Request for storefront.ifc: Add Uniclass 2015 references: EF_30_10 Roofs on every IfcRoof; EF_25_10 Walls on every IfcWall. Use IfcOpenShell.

First a look at what the model holds.

```python
import ifcopenshell

model = ifcopenshell.open("storefront.ifc")
print(model.schema)
print("classifications:", [c.Name for c in model.by_type("IfcClassification")])
for ifc_class in ("IfcDoor", "IfcRoof", "IfcStair", "IfcWall", "IfcWindow"):
    print(ifc_class, len(model.by_type(ifc_class)))
```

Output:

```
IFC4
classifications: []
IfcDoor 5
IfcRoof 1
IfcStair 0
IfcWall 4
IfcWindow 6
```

```python
import ifcopenshell
import ifcopenshell.api.classification

model = ifcopenshell.open("storefront.ifc")

system = ifcopenshell.api.classification.add_classification(model, classification="Uniclass 2015")

codes = {
    "IfcRoof": ("EF_30_10", "Roofs"),
    "IfcWall": ("EF_25_10", "Walls"),
}
for ifc_class, (code, name) in codes.items():
    products = model.by_type(ifc_class)
    ifcopenshell.api.classification.add_reference(
        model, products=products, classification=system, identification=code, name=name
    )
    print(code, len(products))

model.write("storefront-out.ifc")
```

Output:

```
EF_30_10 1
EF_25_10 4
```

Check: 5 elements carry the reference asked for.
